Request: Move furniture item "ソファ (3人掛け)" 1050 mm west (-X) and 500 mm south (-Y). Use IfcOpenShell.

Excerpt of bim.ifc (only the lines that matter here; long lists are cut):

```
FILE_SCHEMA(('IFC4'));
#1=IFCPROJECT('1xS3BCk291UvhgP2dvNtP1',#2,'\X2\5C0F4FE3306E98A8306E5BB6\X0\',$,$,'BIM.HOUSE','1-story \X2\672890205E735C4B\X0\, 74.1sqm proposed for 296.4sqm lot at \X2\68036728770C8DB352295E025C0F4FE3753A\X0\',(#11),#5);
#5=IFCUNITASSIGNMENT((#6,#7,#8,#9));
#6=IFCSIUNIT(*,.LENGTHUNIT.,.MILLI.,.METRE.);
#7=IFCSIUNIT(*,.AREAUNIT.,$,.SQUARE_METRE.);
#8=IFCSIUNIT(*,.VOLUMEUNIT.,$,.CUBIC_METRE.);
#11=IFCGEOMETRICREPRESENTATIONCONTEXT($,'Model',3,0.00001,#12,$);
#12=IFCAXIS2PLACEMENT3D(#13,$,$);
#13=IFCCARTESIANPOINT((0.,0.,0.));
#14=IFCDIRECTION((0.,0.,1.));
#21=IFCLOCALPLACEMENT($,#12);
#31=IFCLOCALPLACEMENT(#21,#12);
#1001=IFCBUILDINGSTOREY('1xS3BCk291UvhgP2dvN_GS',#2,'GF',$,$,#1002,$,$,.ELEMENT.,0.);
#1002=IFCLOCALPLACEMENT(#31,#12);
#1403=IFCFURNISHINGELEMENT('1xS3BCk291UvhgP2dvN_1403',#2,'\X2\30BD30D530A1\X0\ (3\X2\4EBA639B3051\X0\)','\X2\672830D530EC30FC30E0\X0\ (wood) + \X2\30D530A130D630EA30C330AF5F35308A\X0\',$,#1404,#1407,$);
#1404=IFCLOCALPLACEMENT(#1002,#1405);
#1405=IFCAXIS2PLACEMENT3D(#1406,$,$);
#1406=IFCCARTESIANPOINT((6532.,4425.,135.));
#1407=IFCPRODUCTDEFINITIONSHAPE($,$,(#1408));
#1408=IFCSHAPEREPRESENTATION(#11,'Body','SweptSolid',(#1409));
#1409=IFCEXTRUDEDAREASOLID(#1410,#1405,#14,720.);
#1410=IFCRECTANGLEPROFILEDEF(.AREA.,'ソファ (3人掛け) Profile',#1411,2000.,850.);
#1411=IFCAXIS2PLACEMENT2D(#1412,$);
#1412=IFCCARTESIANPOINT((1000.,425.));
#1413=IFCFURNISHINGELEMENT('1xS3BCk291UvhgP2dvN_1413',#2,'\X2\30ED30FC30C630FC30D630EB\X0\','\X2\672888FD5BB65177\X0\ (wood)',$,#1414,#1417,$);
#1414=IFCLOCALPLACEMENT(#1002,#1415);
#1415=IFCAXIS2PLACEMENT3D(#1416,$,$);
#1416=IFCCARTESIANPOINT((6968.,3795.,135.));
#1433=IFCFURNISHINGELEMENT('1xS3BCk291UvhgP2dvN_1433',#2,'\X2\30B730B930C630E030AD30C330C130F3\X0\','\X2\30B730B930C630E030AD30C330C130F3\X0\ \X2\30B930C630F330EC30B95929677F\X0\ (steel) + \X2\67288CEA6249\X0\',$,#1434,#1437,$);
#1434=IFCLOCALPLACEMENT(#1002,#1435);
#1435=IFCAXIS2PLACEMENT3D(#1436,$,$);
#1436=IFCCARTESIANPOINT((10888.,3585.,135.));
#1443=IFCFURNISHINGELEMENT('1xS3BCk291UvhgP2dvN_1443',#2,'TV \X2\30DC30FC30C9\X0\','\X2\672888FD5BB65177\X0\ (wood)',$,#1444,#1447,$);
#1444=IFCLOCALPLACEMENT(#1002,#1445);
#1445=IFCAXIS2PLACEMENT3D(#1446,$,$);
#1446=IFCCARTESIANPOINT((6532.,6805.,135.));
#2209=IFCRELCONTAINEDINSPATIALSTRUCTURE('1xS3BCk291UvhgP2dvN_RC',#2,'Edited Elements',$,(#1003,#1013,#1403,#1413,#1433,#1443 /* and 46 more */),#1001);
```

```python
import ifcopenshell
import ifcopenshell.api.geometry
import ifcopenshell.util.placement
import ifcopenshell.util.unit

model = ifcopenshell.open("bim.ifc")
unit_scale = ifcopenshell.util.unit.calculate_unit_scale(model)

item = model.by_id(1403)
matrix = ifcopenshell.util.placement.get_local_placement(item.ObjectPlacement)
matrix[0, 3] -= 1.05 / unit_scale
matrix[1, 3] -= 0.5 / unit_scale
ifcopenshell.api.geometry.edit_object_placement(model, product=item, matrix=matrix, is_si=False)

print(ifcopenshell.util.placement.get_local_placement(item.ObjectPlacement).round(3) + 0.0)

model.write("bim_rev.ifc")
```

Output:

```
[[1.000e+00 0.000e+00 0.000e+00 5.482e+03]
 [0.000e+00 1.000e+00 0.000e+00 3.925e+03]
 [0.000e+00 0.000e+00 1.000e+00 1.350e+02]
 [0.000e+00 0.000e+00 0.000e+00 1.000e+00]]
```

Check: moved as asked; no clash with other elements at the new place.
